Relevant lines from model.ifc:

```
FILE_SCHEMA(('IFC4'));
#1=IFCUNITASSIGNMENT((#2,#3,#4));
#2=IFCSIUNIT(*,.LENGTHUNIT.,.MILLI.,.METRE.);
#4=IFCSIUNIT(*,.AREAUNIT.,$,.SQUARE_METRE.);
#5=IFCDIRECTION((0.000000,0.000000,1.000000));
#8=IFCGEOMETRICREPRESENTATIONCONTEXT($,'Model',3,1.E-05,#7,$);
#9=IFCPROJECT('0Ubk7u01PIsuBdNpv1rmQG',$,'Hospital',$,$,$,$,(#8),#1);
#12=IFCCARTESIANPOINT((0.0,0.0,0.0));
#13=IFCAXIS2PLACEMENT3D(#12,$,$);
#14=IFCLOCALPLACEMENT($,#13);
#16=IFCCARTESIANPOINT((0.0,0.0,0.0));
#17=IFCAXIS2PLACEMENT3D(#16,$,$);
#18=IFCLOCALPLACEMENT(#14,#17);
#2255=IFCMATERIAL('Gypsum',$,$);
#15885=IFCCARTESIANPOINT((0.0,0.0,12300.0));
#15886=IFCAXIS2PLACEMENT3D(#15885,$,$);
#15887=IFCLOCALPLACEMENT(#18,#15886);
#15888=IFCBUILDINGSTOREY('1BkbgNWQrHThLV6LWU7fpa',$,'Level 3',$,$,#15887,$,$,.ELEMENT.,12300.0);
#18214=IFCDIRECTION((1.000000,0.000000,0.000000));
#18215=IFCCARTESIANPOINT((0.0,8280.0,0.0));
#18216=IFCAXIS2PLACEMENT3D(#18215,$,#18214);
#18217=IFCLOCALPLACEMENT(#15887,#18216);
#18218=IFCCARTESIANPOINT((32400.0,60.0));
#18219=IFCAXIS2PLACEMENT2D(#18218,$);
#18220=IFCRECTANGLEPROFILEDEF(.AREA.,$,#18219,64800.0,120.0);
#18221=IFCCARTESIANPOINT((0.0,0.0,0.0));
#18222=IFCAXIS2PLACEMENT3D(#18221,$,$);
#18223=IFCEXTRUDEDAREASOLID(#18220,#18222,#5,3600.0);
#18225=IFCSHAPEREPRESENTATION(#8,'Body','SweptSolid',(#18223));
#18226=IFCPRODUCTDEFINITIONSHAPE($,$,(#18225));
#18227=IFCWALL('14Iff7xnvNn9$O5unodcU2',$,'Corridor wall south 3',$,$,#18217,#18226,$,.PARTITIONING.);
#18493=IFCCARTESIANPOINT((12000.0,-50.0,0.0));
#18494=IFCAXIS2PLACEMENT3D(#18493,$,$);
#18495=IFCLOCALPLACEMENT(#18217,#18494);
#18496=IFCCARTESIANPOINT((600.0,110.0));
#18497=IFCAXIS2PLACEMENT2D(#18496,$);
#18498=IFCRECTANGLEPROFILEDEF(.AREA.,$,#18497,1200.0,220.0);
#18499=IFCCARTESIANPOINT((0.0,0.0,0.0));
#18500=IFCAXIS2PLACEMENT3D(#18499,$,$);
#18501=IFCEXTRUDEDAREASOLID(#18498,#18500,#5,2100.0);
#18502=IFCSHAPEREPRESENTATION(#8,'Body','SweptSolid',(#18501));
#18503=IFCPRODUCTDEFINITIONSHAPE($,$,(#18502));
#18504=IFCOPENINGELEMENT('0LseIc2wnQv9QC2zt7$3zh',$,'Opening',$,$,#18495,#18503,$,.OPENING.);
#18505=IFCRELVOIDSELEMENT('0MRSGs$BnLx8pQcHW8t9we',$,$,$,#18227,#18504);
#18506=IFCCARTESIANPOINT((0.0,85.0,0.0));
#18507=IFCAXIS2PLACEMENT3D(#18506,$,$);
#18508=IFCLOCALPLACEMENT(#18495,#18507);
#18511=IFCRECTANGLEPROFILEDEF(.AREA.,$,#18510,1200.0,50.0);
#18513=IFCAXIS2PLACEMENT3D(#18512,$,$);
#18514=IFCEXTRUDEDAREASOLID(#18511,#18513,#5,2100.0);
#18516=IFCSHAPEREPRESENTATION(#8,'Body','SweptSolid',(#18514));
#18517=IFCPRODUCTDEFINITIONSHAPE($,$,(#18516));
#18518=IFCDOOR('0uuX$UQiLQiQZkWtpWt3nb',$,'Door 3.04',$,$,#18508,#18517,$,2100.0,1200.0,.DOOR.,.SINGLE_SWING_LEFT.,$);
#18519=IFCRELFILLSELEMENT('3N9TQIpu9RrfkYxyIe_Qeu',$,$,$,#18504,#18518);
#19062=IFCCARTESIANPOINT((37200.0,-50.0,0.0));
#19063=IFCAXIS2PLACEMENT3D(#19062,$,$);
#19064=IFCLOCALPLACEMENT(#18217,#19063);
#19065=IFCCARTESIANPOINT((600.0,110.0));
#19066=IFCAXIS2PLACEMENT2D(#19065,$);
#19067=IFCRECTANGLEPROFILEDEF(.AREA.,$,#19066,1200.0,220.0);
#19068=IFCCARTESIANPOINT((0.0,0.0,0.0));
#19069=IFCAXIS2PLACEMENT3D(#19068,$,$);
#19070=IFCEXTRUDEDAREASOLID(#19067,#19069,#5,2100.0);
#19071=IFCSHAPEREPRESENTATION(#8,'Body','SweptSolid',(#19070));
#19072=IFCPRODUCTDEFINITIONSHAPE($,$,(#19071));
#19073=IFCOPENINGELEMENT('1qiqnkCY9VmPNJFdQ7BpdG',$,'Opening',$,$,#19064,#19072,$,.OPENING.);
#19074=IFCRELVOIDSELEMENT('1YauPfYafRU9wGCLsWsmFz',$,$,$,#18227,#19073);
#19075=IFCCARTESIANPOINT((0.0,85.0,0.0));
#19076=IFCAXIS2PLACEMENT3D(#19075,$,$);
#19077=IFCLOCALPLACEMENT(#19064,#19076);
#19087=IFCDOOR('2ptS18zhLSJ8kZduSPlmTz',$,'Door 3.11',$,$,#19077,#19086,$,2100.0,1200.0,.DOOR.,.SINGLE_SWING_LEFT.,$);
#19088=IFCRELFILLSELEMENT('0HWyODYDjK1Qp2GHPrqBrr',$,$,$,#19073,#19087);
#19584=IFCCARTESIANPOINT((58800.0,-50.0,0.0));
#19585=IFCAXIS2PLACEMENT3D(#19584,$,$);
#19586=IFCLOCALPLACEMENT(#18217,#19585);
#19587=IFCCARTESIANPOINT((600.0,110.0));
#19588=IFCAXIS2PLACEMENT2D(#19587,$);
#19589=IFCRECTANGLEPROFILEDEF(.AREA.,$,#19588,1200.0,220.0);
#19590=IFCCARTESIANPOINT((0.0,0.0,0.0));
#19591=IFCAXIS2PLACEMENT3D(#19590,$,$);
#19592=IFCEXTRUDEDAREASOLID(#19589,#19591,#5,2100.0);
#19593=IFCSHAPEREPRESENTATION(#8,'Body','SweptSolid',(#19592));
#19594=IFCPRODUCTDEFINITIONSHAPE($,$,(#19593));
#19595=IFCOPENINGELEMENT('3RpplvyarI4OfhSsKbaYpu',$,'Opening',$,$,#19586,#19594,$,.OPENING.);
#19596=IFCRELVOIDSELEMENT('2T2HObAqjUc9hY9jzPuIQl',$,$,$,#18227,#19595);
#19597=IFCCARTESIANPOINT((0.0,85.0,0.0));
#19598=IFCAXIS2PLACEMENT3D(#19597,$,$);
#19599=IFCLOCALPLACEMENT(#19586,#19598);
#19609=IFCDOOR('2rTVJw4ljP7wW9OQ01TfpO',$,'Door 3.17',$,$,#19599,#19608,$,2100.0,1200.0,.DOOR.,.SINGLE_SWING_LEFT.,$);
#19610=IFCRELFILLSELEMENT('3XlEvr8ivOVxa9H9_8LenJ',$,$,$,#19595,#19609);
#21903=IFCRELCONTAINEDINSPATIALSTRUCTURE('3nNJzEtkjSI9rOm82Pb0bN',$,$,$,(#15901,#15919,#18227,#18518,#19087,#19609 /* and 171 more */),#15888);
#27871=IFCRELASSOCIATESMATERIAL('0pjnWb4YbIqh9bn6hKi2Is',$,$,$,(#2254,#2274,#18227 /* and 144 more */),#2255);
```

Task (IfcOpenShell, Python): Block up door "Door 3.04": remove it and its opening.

```python
import ifcopenshell
import ifcopenshell.api.feature
import ifcopenshell.api.root
import ifcopenshell.geom
import ifcopenshell.util.shape

model = ifcopenshell.open("model.ifc")
settings = ifcopenshell.geom.settings()


def volume(element):
    """Net volume in cubic metres, openings subtracted."""
    shape = ifcopenshell.geom.create_shape(settings, element)
    return ifcopenshell.util.shape.get_volume(shape.geometry)


door = model.by_guid("0uuX$UQiLQiQZkWtpWt3nb")
opening = door.FillsVoids[0].RelatingOpeningElement
wall = opening.VoidsElements[0].RelatingBuildingElement
before = volume(wall)

ifcopenshell.api.root.remove_product(model, product=door)
ifcopenshell.api.feature.remove_feature(model, feature=opening)

after = volume(wall)

print(f"wall volume {before:.3f} -> {after:.3f} m3")

model.write("model-out.ifc")
```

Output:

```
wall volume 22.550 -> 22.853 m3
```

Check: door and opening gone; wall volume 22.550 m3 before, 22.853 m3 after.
